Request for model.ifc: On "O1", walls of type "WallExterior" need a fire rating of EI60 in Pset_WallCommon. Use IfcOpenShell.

First a look at what the model holds.

```python
import ifcopenshell
import ifcopenshell.util.element

model = ifcopenshell.open("model.ifc")
print(model.schema)
storey = next(s for s in model.by_type("IfcBuildingStorey") if s.Name == "O1")
walls = [e for e in ifcopenshell.util.element.get_decomposition(storey) if e.is_a("IfcWall")]
seen = {}
for e in walls:
    element_type = ifcopenshell.util.element.get_type(e)
    key = (element_type.Name if element_type != e and element_type else None, ifcopenshell.util.element.get_pset(e, "Pset_WallCommon", "FireRating"))
    seen[key] = seen.get(key, 0) + 1
for (name, value), count in sorted(seen.items(), key=str):
    print(count, "x", name, "|", value)
```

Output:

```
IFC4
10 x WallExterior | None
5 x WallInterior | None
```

```python
import ifcopenshell
import ifcopenshell.api.pset
import ifcopenshell.util.element

model = ifcopenshell.open("model.ifc")

storey = next(s for s in model.by_type("IfcBuildingStorey") if s.Name == "O1")
walls = [e for e in ifcopenshell.util.element.get_decomposition(storey) if e.is_a("IfcWall")]

count = 0
for e in walls:
    element_type = ifcopenshell.util.element.get_type(e)
    if element_type in (None, e) or element_type.Name != "WallExterior":
        continue
    # add_pset returns the element's existing set when there is one.
    pset = ifcopenshell.api.pset.add_pset(model, product=e, name="Pset_WallCommon")
    ifcopenshell.api.pset.edit_pset(model, pset=pset, properties={"FireRating": "EI60"})
    count += 1

print(count, "walls updated")

model.write("model_rev.ifc")
```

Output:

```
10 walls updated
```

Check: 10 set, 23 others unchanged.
